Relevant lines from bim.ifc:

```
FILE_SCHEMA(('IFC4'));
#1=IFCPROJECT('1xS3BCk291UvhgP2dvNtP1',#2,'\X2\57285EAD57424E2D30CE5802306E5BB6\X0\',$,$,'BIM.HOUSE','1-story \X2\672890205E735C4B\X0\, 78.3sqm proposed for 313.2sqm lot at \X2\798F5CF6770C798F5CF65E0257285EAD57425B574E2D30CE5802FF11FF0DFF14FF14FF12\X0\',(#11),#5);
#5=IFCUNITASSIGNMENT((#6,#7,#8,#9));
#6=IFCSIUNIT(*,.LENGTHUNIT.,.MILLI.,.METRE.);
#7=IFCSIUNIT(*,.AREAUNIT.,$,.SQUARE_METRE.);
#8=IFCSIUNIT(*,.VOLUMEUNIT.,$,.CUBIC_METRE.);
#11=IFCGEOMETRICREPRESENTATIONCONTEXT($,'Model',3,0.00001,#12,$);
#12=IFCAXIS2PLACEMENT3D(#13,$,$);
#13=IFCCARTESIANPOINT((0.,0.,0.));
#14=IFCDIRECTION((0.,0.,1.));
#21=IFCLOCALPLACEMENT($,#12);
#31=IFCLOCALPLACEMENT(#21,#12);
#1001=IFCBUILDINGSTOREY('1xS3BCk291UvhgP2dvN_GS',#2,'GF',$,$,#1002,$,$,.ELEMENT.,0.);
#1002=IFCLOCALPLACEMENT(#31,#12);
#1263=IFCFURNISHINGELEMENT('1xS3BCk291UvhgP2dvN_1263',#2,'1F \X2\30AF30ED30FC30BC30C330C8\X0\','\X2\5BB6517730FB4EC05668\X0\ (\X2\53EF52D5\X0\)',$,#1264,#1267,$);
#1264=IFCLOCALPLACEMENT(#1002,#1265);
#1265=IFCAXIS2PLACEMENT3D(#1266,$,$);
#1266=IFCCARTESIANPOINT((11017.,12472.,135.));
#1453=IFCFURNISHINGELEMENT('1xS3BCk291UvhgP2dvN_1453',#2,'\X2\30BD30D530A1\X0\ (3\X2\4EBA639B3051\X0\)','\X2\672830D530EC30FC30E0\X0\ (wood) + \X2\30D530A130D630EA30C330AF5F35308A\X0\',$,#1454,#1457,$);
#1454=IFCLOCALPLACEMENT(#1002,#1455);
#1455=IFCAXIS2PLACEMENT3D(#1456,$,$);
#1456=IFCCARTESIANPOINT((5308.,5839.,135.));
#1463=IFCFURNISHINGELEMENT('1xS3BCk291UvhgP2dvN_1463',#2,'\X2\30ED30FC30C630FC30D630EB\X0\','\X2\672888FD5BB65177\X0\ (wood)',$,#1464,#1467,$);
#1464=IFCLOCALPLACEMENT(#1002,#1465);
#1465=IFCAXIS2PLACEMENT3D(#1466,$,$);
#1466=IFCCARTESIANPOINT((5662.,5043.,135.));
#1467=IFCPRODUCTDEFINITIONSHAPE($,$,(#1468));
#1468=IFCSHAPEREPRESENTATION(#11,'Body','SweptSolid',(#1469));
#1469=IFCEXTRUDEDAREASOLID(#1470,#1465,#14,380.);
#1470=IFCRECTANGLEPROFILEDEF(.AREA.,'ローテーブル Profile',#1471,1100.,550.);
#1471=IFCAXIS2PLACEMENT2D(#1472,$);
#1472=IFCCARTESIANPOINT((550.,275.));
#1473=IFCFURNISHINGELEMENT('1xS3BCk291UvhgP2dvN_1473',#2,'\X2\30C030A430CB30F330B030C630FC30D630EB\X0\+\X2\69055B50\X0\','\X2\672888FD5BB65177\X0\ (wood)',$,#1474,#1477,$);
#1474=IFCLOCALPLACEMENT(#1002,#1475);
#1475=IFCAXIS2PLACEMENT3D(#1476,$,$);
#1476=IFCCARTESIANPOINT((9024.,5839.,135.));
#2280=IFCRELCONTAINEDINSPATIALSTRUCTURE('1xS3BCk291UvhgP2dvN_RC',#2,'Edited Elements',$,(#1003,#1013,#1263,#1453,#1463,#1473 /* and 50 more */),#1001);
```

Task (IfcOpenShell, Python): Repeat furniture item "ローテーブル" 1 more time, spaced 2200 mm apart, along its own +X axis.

```python
import ifcopenshell
import ifcopenshell.api.geometry
import ifcopenshell.api.root
import ifcopenshell.util.element
import ifcopenshell.util.placement
import ifcopenshell.util.unit

model = ifcopenshell.open("bim.ifc")
unit_scale = ifcopenshell.util.unit.calculate_unit_scale(model)


def reuse_history(source, copy):
    """copy_class also copies each property set's owner history, people and application; keep the originals."""
    for rel in copy.IsDefinedBy:
        if rel.is_a("IfcRelDefinesByProperties") and (history := rel.RelatingPropertyDefinition.OwnerHistory):
            rel.RelatingPropertyDefinition.OwnerHistory = source.OwnerHistory
            ifcopenshell.util.element.remove_deep2(model, history)


source = model.by_id(1463)
base = ifcopenshell.util.placement.get_local_placement(source.ObjectPlacement)
step = base[:3, 0] * 2.2 / unit_scale

for i in range(1, 2):
    copy = ifcopenshell.api.root.copy_class(model, product=source)
    copy.Representation = ifcopenshell.util.element.copy_deep(
        model, source.Representation, exclude=["IfcGeometricRepresentationContext", "IfcRepresentationMap"]
    )
    reuse_history(source, copy)
    matrix = base.copy()
    matrix[:3, 3] += i * step
    print("added at", matrix[:3, 3].round(3) + 0.0)
    ifcopenshell.api.geometry.edit_object_placement(model, product=copy, matrix=matrix, is_si=False)

model.write("bim-out.ifc")
```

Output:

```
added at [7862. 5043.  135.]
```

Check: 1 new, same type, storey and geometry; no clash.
